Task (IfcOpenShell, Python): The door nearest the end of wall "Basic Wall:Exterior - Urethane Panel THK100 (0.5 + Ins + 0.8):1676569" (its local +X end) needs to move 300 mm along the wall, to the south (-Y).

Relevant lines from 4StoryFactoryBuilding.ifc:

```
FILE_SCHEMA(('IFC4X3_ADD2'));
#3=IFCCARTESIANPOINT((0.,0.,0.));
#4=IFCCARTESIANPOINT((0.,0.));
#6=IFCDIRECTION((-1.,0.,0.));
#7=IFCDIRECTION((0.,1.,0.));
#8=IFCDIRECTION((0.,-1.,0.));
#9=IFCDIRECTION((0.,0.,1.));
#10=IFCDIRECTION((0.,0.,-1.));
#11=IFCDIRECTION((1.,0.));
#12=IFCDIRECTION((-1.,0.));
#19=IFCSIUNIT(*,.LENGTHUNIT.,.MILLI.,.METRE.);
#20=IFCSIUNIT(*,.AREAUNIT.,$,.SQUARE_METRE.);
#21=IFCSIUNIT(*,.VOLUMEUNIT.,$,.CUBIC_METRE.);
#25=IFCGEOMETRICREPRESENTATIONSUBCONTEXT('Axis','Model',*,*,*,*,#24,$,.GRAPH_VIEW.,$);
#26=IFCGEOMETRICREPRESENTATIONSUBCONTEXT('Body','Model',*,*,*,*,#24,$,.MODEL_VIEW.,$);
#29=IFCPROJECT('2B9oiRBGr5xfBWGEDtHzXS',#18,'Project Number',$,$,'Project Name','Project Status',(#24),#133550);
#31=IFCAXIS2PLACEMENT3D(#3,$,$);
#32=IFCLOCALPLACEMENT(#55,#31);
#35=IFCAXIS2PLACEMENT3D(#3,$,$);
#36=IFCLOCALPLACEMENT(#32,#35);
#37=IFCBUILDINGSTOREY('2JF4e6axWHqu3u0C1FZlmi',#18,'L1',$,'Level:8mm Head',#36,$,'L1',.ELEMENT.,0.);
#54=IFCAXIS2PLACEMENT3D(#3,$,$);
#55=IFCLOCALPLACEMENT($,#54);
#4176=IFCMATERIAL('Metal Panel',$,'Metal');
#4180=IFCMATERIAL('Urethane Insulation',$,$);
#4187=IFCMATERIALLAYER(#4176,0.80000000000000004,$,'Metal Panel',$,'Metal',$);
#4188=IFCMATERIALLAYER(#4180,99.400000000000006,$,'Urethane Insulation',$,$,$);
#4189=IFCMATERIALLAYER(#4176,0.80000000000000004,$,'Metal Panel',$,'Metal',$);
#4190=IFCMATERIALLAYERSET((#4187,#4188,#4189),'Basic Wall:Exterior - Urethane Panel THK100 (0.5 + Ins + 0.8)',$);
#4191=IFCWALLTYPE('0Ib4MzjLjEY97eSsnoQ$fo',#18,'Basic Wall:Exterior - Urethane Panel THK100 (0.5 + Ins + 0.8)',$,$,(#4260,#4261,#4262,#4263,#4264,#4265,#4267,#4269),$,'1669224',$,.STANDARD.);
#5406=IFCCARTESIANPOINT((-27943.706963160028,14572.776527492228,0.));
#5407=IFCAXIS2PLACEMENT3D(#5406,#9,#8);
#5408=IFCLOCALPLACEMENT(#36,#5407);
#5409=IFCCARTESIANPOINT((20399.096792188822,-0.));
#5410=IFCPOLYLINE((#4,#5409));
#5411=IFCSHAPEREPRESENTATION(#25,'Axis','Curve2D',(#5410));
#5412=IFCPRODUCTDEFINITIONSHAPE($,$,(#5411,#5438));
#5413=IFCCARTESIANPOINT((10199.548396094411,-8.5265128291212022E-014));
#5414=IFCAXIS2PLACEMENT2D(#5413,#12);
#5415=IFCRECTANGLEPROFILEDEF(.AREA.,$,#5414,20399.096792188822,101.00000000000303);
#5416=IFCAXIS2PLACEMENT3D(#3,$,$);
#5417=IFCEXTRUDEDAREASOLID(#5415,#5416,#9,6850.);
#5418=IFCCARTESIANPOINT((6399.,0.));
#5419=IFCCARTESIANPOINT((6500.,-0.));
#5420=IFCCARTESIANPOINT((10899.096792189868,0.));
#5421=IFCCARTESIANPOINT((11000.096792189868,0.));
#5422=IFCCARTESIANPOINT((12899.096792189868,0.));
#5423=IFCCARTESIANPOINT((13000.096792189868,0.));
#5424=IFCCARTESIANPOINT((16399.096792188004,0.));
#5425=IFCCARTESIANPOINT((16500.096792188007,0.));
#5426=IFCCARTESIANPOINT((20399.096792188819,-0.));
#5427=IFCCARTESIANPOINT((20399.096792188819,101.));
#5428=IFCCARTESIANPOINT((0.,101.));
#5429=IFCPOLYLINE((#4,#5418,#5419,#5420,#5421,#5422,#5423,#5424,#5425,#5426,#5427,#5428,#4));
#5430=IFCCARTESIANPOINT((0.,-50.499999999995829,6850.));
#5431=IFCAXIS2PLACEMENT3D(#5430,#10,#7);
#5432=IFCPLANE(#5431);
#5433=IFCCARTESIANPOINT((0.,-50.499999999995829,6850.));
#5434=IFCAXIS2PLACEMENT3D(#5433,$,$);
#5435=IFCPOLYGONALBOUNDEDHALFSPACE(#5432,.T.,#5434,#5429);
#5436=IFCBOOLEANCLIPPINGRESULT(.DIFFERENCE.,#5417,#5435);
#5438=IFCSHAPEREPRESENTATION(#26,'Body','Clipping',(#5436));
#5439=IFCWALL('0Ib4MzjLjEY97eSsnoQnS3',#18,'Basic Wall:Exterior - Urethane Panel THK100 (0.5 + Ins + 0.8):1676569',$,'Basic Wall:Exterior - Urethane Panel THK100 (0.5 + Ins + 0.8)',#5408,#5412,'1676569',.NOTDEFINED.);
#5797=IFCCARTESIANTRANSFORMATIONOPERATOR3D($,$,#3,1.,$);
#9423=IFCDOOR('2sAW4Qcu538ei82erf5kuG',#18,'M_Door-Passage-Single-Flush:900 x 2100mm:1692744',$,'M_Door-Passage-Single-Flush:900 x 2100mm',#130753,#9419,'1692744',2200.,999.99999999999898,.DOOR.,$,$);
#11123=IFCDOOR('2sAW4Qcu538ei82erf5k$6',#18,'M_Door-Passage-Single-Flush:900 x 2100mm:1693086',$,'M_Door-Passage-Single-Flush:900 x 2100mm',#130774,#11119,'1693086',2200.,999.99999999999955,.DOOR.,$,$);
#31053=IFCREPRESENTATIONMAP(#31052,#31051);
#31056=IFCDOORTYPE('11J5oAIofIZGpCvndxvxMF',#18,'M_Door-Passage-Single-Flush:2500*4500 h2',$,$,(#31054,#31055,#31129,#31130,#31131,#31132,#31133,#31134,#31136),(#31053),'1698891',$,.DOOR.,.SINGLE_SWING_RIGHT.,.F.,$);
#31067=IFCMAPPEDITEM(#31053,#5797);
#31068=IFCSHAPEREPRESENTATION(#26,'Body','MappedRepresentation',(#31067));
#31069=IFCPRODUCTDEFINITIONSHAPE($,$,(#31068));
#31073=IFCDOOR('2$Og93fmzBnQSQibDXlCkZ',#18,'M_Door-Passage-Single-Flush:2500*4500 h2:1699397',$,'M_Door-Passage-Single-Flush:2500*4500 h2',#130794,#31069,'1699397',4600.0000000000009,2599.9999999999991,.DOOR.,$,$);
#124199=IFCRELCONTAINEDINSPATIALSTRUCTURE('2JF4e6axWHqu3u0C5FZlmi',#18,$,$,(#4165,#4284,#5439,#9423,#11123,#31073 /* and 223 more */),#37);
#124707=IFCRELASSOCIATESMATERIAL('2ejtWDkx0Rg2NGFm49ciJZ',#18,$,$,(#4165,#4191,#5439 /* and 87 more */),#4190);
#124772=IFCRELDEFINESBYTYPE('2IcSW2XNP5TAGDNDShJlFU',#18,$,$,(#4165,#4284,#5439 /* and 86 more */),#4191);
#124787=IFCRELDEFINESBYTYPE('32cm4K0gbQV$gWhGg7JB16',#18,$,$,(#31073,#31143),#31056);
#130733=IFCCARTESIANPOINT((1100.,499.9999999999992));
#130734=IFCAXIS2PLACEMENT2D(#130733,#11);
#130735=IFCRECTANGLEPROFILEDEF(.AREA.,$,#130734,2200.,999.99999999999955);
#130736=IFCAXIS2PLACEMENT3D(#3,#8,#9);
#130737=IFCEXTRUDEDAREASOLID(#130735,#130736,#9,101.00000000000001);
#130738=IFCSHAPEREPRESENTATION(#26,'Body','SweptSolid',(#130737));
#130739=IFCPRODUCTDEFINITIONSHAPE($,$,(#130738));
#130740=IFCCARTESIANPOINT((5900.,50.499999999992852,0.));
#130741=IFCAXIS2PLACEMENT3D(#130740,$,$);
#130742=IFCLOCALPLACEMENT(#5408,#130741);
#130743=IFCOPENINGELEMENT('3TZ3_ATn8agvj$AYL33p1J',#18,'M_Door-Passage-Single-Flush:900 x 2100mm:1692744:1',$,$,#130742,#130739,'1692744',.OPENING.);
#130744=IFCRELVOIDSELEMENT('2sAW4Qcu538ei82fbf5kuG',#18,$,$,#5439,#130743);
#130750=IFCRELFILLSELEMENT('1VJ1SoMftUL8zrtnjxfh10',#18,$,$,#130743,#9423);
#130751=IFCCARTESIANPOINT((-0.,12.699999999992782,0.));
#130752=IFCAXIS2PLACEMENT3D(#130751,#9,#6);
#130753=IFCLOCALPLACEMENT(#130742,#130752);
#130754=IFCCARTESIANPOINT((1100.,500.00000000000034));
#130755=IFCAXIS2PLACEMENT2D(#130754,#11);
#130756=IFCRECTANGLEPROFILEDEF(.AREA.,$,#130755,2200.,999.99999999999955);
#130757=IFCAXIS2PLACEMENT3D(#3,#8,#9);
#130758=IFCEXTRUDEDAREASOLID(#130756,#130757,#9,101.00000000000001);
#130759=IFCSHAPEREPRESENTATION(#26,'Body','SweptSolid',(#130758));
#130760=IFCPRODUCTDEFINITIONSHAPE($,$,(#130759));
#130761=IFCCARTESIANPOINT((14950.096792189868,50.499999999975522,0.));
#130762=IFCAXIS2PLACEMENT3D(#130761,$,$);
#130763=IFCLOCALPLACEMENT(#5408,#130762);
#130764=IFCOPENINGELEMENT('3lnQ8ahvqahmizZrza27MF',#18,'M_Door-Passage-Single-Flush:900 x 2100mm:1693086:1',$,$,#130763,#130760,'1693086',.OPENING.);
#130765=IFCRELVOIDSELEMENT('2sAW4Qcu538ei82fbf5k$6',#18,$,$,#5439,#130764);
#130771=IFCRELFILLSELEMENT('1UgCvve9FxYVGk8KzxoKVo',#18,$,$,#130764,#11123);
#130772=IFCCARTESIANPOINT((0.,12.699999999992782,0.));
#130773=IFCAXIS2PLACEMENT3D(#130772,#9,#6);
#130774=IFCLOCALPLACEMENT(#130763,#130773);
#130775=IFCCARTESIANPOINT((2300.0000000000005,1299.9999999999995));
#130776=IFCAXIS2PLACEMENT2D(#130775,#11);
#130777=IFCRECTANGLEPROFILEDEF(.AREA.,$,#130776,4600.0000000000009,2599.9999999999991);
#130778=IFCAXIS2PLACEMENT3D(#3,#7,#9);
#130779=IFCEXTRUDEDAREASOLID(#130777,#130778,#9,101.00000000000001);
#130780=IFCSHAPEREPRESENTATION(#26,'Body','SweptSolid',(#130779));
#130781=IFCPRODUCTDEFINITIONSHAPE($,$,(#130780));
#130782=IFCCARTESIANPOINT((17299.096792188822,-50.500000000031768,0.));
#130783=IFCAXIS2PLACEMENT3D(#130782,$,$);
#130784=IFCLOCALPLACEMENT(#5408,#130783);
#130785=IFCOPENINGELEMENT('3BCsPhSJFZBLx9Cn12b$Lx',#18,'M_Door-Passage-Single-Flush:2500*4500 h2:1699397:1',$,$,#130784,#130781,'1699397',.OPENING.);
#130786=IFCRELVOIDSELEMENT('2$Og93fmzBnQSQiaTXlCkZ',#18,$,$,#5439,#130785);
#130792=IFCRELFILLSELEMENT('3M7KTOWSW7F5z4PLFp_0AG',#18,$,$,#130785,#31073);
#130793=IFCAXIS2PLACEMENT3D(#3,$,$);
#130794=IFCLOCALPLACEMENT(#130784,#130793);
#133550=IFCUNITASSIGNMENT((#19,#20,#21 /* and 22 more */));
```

```python
import ifcopenshell
import ifcopenshell.api.geometry
import ifcopenshell.util.placement
import ifcopenshell.util.unit

model = ifcopenshell.open("4StoryFactoryBuilding.ifc")
unit_scale = ifcopenshell.util.unit.calculate_unit_scale(model)

door = model.by_guid("2$Og93fmzBnQSQibDXlCkZ")
opening = door.FillsVoids[0].RelatingOpeningElement
wall = opening.VoidsElements[0].RelatingBuildingElement

wall_matrix = ifcopenshell.util.placement.get_local_placement(wall.ObjectPlacement)
shift = wall_matrix[:3, 0] * 0.3 / unit_scale
before = ifcopenshell.util.placement.get_local_placement(door.ObjectPlacement)[:3, 3].copy()

# The door is placed relative to its opening, so it follows when the opening moves.
matrix = ifcopenshell.util.placement.get_local_placement(opening.ObjectPlacement)
matrix[:3, 3] += shift
ifcopenshell.api.geometry.edit_object_placement(
    model, product=opening, matrix=matrix, is_si=False, should_transform_children=True
)

after = ifcopenshell.util.placement.get_local_placement(door.ObjectPlacement)[:3, 3]
print("door moved by", (after - before).round(3) + 0.0)

model.write("4StoryFactoryBuilding_v2.ifc")
```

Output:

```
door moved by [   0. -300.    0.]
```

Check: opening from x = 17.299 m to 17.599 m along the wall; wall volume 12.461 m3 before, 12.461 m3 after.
